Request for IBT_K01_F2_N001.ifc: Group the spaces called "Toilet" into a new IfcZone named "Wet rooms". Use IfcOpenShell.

First a look at what the model holds.

```python
import ifcopenshell

model = ifcopenshell.open("IBT_K01_F2_N001.ifc")
print(model.schema)
seen = {}
for space in model.by_type("IfcSpace"):
    seen[space.LongName] = seen.get(space.LongName, 0) + 1
for name, count in sorted(seen.items(), key=str):
    print(count, "x", name)
print("zones:", [z.Name for z in model.by_type("IfcZone")][:20])
```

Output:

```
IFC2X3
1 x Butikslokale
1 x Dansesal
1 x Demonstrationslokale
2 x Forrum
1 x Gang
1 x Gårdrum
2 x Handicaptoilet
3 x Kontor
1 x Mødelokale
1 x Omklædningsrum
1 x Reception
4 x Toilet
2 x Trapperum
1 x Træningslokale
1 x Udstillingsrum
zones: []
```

```python
import ifcopenshell
import ifcopenshell.api.group
import ifcopenshell.api.root

model = ifcopenshell.open("IBT_K01_F2_N001.ifc")

names = {"Toilet"}
spaces = [s for s in model.by_type("IfcSpace") if s.LongName in names]

zone = ifcopenshell.api.root.create_entity(model, ifc_class="IfcZone", name="Wet rooms")
ifcopenshell.api.group.assign_group(model, products=spaces, group=zone)
print(len(spaces), "spaces in", zone.Name)

model.write("IBT_K01_F2_N001_rev.ifc")
```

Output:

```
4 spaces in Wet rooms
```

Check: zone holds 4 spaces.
